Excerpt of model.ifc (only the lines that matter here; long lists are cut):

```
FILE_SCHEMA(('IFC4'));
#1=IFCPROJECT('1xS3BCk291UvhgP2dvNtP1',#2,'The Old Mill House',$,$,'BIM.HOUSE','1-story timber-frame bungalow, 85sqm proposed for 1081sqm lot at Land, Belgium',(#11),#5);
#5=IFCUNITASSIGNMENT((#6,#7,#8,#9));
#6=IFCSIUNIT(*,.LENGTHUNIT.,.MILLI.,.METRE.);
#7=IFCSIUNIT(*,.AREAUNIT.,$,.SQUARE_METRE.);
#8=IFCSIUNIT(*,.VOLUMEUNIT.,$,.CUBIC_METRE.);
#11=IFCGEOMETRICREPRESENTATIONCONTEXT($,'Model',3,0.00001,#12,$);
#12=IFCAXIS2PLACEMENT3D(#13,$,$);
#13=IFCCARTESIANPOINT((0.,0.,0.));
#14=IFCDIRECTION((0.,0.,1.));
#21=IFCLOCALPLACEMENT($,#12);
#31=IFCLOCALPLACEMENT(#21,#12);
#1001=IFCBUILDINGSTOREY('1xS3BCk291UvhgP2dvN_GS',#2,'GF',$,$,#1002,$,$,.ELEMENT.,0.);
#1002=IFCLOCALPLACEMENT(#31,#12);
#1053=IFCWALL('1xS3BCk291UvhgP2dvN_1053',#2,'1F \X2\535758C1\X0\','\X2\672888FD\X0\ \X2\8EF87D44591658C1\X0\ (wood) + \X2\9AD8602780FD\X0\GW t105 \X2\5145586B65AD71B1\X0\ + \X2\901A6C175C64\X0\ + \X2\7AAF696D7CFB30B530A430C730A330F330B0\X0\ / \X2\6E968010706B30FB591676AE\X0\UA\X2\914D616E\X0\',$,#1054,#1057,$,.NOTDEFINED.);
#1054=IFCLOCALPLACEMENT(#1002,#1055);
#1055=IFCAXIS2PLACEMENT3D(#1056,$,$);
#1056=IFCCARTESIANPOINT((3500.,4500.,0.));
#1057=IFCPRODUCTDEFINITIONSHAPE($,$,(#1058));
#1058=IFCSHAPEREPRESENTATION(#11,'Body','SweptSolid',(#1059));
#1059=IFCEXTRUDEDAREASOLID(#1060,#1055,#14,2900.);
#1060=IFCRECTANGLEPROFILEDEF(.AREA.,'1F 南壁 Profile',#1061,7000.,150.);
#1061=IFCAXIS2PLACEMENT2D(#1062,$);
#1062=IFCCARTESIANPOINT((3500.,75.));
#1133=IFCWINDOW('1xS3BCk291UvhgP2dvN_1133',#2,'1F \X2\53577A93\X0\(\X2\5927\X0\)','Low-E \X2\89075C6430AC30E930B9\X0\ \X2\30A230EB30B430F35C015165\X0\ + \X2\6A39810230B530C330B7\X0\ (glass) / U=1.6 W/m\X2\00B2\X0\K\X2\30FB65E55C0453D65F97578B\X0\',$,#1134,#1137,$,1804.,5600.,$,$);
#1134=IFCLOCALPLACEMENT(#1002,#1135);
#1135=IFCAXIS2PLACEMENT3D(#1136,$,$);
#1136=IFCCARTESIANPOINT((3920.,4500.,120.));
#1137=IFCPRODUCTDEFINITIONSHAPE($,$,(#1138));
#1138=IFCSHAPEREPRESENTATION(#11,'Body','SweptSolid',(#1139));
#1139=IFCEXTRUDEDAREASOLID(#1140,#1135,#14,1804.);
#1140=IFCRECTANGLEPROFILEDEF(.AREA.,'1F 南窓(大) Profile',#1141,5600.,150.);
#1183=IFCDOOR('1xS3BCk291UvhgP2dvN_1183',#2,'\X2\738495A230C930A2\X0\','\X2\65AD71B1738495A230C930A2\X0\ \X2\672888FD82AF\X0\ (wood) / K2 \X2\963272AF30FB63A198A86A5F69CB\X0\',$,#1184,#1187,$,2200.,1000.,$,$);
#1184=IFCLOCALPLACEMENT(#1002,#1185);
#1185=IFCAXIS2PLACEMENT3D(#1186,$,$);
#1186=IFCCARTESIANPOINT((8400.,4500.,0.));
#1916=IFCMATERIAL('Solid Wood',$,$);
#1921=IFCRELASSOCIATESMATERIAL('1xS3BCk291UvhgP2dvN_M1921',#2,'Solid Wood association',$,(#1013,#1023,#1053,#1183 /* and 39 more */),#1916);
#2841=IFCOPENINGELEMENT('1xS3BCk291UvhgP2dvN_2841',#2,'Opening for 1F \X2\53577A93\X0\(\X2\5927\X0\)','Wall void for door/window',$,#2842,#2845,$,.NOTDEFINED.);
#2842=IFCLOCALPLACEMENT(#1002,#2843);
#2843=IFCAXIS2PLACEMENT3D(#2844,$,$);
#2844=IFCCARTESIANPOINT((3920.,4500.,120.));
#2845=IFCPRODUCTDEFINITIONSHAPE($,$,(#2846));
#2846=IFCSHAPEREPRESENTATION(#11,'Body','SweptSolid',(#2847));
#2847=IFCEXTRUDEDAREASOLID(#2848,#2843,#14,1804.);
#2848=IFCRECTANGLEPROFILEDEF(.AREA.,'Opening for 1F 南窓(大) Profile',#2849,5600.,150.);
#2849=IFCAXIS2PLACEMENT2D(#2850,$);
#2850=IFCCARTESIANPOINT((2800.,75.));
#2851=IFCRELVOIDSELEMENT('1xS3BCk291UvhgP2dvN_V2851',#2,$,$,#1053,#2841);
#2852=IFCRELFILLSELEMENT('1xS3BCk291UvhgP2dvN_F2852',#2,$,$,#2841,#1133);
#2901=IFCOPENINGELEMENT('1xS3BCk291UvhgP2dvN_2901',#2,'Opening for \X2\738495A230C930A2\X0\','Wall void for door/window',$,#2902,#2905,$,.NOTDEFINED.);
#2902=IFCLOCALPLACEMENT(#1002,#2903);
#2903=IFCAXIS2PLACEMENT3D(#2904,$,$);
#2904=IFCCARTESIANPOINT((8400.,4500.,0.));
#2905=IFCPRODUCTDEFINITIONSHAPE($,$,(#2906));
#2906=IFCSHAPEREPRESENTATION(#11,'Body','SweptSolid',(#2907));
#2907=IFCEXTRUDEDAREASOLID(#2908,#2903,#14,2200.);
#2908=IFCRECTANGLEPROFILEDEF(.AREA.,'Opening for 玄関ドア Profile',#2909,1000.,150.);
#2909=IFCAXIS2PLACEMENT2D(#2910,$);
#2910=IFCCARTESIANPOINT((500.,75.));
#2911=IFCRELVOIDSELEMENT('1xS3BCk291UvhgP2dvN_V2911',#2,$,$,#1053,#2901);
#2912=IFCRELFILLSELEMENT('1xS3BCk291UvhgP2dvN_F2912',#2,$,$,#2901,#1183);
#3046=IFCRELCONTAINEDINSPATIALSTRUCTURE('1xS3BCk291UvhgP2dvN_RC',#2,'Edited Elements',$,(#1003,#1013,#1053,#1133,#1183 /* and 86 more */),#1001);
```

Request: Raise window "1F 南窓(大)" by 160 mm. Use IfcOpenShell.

```python
import numpy as np
import ifcopenshell
import ifcopenshell.api.geometry
import ifcopenshell.util.placement
import ifcopenshell.util.unit

model = ifcopenshell.open("model.ifc")
unit_scale = ifcopenshell.util.unit.calculate_unit_scale(model)

window = model.by_id(1133)
opening = window.FillsVoids[0].RelatingOpeningElement
dz = 160.0

shift = np.array([0.0, 0.0, dz])
# The window is not placed relative to its opening, so move both.
for product in (opening, window):
    matrix = ifcopenshell.util.placement.get_local_placement(product.ObjectPlacement)
    matrix[:3, 3] += shift
    ifcopenshell.api.geometry.edit_object_placement(model, product=product, matrix=matrix, is_si=False)

print(f"moved by {dz * unit_scale:+.3f} m")

model.write("model-out.ifc")
```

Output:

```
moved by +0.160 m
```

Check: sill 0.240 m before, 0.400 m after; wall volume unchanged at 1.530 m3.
